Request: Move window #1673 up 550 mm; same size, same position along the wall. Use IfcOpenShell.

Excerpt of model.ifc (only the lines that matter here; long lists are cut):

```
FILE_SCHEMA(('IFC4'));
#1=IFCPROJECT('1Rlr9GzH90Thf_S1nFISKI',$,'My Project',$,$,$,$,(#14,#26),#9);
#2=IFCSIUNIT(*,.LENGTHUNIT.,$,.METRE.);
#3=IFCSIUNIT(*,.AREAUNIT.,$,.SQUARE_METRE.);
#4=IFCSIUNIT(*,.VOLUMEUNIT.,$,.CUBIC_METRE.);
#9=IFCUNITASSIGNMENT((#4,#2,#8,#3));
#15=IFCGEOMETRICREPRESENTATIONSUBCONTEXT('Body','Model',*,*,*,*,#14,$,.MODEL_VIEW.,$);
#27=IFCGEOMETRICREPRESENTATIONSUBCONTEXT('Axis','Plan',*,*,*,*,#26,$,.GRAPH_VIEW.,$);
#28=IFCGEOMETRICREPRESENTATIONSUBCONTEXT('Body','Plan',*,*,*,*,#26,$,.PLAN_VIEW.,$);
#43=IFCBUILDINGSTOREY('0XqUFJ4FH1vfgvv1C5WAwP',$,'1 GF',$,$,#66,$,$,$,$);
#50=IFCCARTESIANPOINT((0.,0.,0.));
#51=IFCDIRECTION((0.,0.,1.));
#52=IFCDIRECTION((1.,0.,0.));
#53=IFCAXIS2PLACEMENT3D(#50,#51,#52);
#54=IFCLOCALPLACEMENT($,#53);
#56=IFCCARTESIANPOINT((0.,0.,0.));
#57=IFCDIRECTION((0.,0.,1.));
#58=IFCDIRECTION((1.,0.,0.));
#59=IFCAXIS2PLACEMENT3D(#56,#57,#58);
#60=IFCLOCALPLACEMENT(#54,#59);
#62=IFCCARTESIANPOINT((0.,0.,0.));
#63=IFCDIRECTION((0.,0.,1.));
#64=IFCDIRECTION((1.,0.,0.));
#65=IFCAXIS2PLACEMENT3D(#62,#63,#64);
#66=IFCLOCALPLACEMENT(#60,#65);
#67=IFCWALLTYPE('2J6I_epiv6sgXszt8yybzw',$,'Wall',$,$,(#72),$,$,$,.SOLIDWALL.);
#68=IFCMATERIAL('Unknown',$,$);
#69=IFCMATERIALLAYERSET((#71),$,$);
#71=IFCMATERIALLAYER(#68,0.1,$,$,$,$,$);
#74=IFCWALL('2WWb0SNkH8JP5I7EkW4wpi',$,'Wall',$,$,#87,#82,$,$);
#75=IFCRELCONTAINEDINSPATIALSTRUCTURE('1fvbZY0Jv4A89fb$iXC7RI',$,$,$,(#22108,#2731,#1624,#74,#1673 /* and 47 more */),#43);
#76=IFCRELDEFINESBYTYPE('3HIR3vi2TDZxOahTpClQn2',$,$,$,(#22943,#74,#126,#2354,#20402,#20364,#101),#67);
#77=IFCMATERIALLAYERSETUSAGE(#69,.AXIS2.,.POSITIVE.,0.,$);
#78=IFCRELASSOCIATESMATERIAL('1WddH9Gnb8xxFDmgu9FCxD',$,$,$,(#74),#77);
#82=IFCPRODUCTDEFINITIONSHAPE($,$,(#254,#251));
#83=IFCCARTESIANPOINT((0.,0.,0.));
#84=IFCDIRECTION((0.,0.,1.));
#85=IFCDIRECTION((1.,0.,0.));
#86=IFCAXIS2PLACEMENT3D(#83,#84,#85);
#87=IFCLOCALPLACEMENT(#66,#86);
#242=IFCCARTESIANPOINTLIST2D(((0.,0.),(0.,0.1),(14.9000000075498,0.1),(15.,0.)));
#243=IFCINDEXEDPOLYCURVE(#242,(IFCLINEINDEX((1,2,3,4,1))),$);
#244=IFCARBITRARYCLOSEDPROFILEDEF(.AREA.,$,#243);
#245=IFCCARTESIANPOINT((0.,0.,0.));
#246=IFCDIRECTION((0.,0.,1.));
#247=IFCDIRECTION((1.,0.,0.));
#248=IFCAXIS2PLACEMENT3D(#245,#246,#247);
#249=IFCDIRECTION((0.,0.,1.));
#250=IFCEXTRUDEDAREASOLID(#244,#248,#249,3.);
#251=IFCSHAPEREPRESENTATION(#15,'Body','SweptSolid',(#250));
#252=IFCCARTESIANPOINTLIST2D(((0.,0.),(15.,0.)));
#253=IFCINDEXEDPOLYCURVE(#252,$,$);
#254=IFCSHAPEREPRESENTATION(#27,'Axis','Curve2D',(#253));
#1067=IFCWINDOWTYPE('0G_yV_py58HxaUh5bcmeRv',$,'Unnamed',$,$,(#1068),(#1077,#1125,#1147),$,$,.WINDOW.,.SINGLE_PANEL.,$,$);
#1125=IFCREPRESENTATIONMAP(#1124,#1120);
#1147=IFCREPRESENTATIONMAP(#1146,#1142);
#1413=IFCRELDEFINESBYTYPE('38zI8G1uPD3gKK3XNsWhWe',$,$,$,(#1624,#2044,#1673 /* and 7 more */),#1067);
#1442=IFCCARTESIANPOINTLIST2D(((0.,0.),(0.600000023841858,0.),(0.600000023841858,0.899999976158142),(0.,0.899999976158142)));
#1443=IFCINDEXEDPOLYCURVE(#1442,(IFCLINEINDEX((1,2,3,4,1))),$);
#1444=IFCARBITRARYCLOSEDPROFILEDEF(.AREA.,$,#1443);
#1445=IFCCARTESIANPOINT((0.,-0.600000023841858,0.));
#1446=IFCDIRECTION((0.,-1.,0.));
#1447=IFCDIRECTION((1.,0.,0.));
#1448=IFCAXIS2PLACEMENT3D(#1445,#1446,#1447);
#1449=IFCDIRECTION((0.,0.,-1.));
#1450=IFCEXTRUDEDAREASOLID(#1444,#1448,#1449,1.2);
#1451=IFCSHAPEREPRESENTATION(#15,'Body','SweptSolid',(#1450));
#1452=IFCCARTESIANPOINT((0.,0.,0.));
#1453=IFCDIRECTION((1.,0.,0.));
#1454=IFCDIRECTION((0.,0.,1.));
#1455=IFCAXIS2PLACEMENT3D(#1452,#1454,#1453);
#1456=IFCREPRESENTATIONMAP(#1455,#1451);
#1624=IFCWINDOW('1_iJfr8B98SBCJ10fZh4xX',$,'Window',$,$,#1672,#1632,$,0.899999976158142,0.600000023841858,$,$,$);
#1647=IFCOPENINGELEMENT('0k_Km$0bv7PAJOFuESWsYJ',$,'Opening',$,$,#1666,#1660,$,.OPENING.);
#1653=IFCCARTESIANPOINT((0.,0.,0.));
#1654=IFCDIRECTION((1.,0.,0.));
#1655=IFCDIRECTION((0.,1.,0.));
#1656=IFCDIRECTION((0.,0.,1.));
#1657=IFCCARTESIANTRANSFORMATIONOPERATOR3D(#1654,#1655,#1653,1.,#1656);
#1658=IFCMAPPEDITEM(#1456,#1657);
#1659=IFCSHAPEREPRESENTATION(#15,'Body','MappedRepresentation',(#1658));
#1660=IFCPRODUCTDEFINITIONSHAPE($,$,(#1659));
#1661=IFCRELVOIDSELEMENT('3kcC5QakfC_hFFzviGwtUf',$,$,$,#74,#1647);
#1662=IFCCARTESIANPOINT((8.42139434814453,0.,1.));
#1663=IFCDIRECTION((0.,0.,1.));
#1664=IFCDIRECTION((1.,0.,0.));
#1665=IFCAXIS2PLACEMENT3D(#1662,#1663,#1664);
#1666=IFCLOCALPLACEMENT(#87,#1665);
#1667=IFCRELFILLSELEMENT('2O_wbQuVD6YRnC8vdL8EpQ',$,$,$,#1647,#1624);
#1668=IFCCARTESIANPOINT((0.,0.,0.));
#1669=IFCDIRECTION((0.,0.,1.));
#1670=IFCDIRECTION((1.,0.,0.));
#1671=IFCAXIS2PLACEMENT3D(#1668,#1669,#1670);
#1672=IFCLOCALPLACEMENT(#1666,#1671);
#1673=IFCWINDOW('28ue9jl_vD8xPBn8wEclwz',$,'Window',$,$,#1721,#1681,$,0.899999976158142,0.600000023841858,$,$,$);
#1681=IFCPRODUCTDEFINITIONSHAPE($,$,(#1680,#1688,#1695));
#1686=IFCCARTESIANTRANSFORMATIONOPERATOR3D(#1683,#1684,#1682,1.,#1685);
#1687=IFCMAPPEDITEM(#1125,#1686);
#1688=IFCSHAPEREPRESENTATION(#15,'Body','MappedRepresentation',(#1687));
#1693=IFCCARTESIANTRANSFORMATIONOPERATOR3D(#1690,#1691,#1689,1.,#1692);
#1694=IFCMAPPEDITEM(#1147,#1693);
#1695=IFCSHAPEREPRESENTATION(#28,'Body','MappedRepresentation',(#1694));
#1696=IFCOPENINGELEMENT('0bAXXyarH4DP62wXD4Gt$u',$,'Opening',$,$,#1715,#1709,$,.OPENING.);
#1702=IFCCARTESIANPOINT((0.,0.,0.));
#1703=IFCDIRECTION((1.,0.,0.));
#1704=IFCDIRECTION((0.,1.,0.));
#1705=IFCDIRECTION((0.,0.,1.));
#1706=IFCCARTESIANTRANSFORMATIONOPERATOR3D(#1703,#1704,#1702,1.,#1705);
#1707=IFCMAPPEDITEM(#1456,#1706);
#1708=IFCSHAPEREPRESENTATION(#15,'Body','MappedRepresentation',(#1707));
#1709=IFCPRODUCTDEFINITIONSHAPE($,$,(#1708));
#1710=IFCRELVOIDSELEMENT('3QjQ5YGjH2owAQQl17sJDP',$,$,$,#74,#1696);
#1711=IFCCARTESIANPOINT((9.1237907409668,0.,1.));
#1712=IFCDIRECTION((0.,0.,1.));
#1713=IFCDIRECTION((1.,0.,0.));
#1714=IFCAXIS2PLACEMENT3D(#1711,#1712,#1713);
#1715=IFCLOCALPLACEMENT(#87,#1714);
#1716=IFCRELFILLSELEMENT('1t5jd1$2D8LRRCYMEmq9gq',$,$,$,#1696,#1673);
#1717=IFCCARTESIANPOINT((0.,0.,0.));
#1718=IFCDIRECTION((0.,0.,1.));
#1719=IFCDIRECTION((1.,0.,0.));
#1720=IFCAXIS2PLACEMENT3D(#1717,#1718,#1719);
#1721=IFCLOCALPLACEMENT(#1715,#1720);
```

```python
import numpy as np
import ifcopenshell
import ifcopenshell.api.geometry
import ifcopenshell.util.placement
import ifcopenshell.util.unit

model = ifcopenshell.open("model.ifc")
unit_scale = ifcopenshell.util.unit.calculate_unit_scale(model)

window = model.by_id(1673)
opening = window.FillsVoids[0].RelatingOpeningElement
dz = 0.55 / unit_scale

shift = np.array([0.0, 0.0, dz])
# The window is placed relative to its opening, so it follows when the opening moves.
matrix = ifcopenshell.util.placement.get_local_placement(opening.ObjectPlacement)
matrix[:3, 3] += shift
ifcopenshell.api.geometry.edit_object_placement(
    model, product=opening, matrix=matrix, is_si=False, should_transform_children=True
)

print(f"moved by {dz * unit_scale:+.3f} m")

model.write("model_updated.ifc")
```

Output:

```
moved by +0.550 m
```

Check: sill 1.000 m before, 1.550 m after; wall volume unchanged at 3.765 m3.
